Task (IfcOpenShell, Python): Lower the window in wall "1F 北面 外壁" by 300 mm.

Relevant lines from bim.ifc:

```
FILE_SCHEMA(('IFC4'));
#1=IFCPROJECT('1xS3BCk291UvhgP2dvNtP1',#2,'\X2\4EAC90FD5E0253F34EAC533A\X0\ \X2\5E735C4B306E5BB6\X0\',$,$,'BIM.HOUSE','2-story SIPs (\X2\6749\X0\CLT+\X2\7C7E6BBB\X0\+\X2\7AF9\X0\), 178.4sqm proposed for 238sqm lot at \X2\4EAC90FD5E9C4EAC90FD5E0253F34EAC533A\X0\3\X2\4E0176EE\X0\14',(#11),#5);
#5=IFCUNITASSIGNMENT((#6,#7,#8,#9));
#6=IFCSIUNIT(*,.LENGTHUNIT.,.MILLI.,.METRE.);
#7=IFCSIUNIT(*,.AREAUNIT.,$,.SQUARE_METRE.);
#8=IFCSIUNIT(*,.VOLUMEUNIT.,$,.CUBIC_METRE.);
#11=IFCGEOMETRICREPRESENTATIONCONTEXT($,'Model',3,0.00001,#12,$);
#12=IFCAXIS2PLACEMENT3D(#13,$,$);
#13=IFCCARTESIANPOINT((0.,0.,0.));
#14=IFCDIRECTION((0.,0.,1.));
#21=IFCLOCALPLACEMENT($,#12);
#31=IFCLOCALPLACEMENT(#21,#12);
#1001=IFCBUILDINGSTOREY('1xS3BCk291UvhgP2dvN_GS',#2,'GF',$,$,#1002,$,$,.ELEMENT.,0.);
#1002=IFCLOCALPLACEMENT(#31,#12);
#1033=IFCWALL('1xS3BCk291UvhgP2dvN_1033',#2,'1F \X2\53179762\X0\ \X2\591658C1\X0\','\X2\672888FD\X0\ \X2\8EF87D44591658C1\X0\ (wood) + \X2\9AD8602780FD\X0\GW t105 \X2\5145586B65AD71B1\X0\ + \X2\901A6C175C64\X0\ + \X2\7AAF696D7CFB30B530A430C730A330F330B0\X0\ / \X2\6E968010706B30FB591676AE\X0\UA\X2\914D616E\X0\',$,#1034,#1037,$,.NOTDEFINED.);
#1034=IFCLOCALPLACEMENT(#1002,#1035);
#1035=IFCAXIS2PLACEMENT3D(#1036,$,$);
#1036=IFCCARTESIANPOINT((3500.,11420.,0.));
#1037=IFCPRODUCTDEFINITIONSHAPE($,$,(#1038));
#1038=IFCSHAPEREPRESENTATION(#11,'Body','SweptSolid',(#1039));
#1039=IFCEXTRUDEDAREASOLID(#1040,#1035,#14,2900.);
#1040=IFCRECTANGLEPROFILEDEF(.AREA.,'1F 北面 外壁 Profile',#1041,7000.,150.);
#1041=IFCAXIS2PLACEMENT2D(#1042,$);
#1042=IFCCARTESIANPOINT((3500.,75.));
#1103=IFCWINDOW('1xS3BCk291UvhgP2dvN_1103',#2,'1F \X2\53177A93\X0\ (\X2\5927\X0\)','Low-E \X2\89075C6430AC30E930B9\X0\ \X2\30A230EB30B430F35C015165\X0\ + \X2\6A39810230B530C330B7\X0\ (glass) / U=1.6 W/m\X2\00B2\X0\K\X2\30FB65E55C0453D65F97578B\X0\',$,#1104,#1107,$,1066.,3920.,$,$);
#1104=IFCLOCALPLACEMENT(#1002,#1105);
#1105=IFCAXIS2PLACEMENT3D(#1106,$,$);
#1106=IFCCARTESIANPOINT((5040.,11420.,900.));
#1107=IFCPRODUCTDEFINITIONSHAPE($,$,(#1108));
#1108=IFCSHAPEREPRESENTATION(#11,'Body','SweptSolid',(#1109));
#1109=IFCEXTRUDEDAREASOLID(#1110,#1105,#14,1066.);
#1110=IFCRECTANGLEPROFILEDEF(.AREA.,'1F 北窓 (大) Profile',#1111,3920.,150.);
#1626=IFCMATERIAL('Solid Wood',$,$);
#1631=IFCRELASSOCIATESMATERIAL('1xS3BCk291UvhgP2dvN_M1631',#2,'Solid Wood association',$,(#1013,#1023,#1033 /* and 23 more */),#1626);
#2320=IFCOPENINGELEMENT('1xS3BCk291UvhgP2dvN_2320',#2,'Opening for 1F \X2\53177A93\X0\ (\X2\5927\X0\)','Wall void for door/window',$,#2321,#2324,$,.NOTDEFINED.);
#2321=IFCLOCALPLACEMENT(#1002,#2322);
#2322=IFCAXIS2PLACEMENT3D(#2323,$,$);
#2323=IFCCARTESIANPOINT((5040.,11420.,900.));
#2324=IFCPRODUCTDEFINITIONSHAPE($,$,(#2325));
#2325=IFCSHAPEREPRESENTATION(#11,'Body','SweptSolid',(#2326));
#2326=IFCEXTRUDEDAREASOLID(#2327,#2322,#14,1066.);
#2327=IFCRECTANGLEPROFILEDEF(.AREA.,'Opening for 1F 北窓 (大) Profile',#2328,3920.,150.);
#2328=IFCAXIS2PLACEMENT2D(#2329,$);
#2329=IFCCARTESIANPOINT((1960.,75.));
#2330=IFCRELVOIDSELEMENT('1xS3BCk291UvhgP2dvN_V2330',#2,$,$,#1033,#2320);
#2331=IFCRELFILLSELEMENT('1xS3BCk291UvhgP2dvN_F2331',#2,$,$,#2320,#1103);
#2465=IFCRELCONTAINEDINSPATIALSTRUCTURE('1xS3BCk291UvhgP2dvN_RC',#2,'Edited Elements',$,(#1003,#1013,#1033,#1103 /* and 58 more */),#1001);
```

```python
import numpy as np
import ifcopenshell
import ifcopenshell.api.geometry
import ifcopenshell.util.placement
import ifcopenshell.util.unit

model = ifcopenshell.open("bim.ifc")
unit_scale = ifcopenshell.util.unit.calculate_unit_scale(model)

window = model.by_guid("1xS3BCk291UvhgP2dvN_1103")
opening = window.FillsVoids[0].RelatingOpeningElement
dz = -300.0

shift = np.array([0.0, 0.0, dz])
# The window is not placed relative to its opening, so move both.
for product in (opening, window):
    matrix = ifcopenshell.util.placement.get_local_placement(product.ObjectPlacement)
    matrix[:3, 3] += shift
    ifcopenshell.api.geometry.edit_object_placement(model, product=product, matrix=matrix, is_si=False)

print(f"moved by {dz * unit_scale:+.3f} m")

model.write("bim_v2.ifc")
```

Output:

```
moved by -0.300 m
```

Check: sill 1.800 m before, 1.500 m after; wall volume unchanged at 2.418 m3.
